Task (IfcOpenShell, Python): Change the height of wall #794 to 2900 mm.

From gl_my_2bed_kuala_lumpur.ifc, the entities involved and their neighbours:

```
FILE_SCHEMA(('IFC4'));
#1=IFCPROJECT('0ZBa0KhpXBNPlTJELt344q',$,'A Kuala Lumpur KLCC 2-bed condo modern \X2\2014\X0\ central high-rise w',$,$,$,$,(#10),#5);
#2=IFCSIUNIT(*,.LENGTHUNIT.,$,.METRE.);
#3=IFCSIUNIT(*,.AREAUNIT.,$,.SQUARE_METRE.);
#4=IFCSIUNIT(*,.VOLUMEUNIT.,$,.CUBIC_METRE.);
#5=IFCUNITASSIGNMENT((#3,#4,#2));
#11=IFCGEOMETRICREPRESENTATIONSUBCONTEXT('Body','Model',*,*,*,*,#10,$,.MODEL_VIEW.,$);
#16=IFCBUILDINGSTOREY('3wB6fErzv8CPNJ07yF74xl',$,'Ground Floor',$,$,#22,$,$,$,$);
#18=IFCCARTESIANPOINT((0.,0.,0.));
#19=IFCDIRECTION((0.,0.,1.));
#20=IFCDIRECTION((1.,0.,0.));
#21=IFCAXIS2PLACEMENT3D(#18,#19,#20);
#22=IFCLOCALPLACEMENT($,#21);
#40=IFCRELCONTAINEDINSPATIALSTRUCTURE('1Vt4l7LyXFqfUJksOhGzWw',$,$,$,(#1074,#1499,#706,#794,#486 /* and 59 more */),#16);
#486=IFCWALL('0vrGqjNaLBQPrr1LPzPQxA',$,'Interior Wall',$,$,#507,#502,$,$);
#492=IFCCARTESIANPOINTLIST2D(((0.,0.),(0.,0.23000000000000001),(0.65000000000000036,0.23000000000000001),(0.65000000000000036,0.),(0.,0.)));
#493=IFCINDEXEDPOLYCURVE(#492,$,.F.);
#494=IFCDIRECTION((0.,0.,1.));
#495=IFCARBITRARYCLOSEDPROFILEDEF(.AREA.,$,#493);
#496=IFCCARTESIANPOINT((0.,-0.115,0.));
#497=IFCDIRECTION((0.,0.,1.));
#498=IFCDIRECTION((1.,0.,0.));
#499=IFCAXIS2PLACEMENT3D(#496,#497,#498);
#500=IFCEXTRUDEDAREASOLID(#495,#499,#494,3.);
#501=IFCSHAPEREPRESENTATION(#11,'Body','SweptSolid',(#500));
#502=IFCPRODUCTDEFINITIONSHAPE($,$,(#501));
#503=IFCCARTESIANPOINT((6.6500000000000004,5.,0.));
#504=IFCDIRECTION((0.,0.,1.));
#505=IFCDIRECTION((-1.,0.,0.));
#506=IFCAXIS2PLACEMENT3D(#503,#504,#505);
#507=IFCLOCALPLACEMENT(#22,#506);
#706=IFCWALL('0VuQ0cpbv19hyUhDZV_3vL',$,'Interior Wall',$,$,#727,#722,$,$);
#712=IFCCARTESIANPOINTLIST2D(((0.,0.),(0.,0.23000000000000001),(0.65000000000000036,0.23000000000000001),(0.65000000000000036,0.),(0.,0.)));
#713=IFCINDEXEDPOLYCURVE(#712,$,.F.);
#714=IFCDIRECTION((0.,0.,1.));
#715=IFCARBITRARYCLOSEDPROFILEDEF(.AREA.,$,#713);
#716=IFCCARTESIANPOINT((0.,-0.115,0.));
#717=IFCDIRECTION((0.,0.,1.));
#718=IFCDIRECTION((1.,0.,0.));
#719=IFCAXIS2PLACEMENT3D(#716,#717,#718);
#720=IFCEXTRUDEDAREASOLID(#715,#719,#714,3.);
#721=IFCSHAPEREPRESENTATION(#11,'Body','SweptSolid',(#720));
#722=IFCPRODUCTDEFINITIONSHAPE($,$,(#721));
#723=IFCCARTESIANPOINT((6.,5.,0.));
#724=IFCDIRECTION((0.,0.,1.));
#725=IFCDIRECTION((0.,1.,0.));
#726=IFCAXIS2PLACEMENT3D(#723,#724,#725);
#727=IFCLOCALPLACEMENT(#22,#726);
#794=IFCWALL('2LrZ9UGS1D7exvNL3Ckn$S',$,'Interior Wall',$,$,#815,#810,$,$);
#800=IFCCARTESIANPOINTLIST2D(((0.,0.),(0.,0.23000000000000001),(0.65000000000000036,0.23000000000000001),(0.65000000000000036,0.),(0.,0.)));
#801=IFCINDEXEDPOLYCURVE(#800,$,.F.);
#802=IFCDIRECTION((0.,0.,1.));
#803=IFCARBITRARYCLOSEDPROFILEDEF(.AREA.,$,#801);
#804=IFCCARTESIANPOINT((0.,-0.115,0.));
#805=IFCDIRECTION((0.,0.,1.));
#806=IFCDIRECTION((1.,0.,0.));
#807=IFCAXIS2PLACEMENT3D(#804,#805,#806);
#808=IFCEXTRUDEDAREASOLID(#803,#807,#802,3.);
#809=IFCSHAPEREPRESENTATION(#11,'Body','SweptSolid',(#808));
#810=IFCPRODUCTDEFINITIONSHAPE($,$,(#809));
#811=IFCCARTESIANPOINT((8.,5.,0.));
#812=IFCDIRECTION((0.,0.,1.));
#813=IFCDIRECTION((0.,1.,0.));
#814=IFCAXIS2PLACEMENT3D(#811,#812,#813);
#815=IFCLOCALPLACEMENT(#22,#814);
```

```python
import ifcopenshell
import ifcopenshell.geom
import ifcopenshell.util.representation
import ifcopenshell.util.shape
import ifcopenshell.util.unit

model = ifcopenshell.open("gl_my_2bed_kuala_lumpur.ifc")
unit_scale = ifcopenshell.util.unit.calculate_unit_scale(model)
settings = ifcopenshell.geom.settings()


def volume(element):
    """Net volume in cubic metres, openings subtracted."""
    shape = ifcopenshell.geom.create_shape(settings, element)
    return ifcopenshell.util.shape.get_volume(shape.geometry)


wall = model.by_id(794)
before = volume(wall)

body = ifcopenshell.util.representation.get_representation(wall, "Model", "Body")
solid = body.Items[0]
old_height = solid.Depth
solid.Depth = 2.9 / unit_scale
after = volume(wall)

print(f"height {old_height:g} -> {solid.Depth:g}, volume {before:.3f} -> {after:.3f} m3")

model.write("gl_my_2bed_kuala_lumpur_updated.ifc")
```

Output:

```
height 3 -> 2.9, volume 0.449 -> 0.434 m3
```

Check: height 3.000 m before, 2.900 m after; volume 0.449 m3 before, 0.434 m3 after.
